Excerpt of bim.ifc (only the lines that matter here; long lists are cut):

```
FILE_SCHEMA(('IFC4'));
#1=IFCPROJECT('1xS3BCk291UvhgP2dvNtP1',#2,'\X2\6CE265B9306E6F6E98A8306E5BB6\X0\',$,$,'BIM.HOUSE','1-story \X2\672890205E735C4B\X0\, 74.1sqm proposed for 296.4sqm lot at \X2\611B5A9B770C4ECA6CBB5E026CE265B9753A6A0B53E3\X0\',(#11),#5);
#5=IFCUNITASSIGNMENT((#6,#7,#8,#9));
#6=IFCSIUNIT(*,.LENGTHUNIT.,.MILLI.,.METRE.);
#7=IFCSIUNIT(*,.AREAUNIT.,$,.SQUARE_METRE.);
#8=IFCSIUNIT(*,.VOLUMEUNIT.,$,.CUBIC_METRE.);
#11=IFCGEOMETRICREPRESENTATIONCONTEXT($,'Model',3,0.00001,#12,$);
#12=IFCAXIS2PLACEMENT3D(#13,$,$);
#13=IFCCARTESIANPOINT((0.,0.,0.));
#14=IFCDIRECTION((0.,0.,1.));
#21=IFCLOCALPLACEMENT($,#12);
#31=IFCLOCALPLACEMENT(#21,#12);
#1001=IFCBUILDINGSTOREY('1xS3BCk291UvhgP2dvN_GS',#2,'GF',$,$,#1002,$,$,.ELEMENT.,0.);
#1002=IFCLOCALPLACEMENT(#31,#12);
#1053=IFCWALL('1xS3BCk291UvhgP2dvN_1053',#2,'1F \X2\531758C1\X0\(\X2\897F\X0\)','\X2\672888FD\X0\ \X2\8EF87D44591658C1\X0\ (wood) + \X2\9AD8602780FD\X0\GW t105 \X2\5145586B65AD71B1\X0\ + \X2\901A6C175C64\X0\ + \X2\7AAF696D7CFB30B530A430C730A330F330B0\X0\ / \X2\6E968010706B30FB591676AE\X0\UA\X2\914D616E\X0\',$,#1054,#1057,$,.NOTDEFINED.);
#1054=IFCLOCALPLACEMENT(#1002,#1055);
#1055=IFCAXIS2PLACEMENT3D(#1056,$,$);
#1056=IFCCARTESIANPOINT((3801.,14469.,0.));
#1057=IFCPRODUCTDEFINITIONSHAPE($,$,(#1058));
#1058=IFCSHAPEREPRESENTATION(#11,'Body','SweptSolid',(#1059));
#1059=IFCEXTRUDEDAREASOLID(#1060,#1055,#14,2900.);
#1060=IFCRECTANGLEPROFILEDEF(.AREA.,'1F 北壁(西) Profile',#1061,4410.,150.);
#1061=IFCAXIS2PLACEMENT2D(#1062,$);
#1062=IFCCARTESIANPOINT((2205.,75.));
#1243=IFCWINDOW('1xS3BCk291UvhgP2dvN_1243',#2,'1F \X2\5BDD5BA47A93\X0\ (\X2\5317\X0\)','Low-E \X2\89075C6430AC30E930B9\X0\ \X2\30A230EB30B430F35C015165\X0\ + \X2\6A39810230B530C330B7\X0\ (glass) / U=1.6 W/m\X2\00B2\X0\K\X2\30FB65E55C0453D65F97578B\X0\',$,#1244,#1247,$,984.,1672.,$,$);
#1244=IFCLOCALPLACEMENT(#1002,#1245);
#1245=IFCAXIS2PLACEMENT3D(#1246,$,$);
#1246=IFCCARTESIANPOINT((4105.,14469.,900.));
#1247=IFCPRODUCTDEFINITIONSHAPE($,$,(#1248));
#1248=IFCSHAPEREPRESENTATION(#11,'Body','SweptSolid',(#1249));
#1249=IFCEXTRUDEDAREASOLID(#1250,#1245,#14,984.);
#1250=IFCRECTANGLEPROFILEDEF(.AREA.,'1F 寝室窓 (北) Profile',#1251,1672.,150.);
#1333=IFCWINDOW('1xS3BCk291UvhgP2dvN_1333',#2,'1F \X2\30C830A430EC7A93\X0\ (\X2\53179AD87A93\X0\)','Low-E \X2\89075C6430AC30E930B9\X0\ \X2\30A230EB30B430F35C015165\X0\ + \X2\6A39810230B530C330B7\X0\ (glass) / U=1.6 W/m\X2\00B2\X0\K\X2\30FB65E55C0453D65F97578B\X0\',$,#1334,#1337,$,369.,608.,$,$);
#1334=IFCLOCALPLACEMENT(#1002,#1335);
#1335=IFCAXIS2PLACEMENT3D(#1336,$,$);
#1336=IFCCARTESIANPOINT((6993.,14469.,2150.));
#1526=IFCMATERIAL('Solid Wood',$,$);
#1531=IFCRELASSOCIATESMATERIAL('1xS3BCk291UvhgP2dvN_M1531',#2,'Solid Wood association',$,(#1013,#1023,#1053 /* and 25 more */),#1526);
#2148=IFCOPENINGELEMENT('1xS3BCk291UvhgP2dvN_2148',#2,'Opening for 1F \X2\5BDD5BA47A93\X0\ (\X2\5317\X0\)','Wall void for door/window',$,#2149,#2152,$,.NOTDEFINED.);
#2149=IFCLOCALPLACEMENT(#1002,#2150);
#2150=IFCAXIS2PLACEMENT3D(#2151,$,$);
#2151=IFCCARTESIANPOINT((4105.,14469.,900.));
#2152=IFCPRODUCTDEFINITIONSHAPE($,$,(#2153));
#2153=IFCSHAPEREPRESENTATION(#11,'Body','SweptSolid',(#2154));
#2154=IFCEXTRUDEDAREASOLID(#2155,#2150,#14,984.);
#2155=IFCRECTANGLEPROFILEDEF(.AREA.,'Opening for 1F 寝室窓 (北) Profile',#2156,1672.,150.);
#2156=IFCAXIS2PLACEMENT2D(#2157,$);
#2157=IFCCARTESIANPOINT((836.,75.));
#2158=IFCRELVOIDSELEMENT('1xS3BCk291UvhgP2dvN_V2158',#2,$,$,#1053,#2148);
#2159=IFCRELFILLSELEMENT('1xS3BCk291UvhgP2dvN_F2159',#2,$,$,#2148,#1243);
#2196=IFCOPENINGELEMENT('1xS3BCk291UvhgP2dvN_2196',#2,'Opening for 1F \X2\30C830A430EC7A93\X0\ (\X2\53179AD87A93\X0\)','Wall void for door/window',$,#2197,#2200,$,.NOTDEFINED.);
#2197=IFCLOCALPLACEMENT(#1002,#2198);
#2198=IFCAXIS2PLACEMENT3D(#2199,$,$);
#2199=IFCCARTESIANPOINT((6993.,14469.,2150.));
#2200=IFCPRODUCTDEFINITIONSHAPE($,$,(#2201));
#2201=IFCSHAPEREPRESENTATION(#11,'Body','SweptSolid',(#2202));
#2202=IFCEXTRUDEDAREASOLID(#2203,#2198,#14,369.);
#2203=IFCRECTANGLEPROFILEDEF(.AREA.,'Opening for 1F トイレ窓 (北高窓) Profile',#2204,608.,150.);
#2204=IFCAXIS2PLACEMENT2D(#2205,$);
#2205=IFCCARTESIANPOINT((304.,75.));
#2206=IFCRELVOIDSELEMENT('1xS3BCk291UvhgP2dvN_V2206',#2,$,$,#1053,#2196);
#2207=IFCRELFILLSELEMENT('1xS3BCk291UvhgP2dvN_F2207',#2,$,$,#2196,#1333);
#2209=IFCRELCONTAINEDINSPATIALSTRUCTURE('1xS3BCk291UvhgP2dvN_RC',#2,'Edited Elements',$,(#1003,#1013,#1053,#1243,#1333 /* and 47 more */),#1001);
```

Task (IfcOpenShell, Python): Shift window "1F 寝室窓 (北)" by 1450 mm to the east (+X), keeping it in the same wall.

```python
import ifcopenshell
import ifcopenshell.api.geometry
import ifcopenshell.util.placement
import ifcopenshell.util.unit

model = ifcopenshell.open("bim.ifc")
unit_scale = ifcopenshell.util.unit.calculate_unit_scale(model)

window = model.by_guid("1xS3BCk291UvhgP2dvN_1243")
opening = window.FillsVoids[0].RelatingOpeningElement
wall = opening.VoidsElements[0].RelatingBuildingElement

wall_matrix = ifcopenshell.util.placement.get_local_placement(wall.ObjectPlacement)
shift = wall_matrix[:3, 0] * 1.45 / unit_scale
before = ifcopenshell.util.placement.get_local_placement(window.ObjectPlacement)[:3, 3].copy()

# The window is not placed relative to its opening, so move both.
for product in (opening, window):
    matrix = ifcopenshell.util.placement.get_local_placement(product.ObjectPlacement)
    matrix[:3, 3] += shift
    ifcopenshell.api.geometry.edit_object_placement(model, product=product, matrix=matrix, is_si=False)

after = ifcopenshell.util.placement.get_local_placement(window.ObjectPlacement)[:3, 3]
print("window moved by", (after - before).round(3) + 0.0)

model.write("bim_rev.ifc")
```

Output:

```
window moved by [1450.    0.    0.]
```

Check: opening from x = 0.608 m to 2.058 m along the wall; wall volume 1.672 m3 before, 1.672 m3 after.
